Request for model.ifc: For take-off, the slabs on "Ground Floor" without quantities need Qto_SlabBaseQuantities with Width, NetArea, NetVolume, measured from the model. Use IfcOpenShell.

First a look at what the model holds.

```python
import ifcopenshell
import ifcopenshell.util.element
import ifcopenshell.util.unit

model = ifcopenshell.open("model.ifc")
print(model.schema)
for unit_type in ("LENGTHUNIT", "AREAUNIT", "VOLUMEUNIT"):
    print(unit_type, ifcopenshell.util.unit.calculate_unit_scale(model, unit_type))
storey = next(s for s in model.by_type("IfcBuildingStorey") if s.Name == "Ground Floor")
slabs = [e for e in ifcopenshell.util.element.get_decomposition(storey) if e.is_a("IfcSlab")]
for e in sorted(slabs, key=lambda e: e.id()):
    print(e.id(), e.is_a(), e.Name, list(ifcopenshell.util.element.get_psets(e, qtos_only=True)), sep=" | ")
```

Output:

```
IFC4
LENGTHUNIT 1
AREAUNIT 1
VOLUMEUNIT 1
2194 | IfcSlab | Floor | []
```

```python
import ifcopenshell
import ifcopenshell.api.pset
import ifcopenshell.geom
import ifcopenshell.util.element
import ifcopenshell.util.shape
import ifcopenshell.util.unit

model = ifcopenshell.open("model.ifc")
unit_scale = ifcopenshell.util.unit.calculate_unit_scale(model)
area_scale = ifcopenshell.util.unit.calculate_unit_scale(model, "AREAUNIT")
volume_scale = ifcopenshell.util.unit.calculate_unit_scale(model, "VOLUMEUNIT")
settings = ifcopenshell.geom.settings()

storey = next(s for s in model.by_type("IfcBuildingStorey") if s.Name == "Ground Floor")
slabs = [e for e in ifcopenshell.util.element.get_decomposition(storey) if e.is_a("IfcSlab")]

for e in sorted(slabs, key=lambda e: e.id()):
    if ifcopenshell.util.element.get_psets(e, qtos_only=True, should_inherit=False):
        continue
    # Geometry comes back in metres, in the element's own axes.
    shape = ifcopenshell.geom.create_shape(settings, e)
    values = {
        "Width": ifcopenshell.util.shape.get_z(shape.geometry) / unit_scale,
        "NetArea": ifcopenshell.util.shape.get_footprint_area(shape.geometry) / area_scale,
        "NetVolume": ifcopenshell.util.shape.get_volume(shape.geometry) / volume_scale,
    }
    qto = ifcopenshell.api.pset.add_qto(model, product=e, name="Qto_SlabBaseQuantities")
    ifcopenshell.api.pset.edit_qto(model, qto=qto, properties=values)
    print(e.id(), {k: round(v, 3) for k, v in values.items()})

model.write("model_rev.ifc")
```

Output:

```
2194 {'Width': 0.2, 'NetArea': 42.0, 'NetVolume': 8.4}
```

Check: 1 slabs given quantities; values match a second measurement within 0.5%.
